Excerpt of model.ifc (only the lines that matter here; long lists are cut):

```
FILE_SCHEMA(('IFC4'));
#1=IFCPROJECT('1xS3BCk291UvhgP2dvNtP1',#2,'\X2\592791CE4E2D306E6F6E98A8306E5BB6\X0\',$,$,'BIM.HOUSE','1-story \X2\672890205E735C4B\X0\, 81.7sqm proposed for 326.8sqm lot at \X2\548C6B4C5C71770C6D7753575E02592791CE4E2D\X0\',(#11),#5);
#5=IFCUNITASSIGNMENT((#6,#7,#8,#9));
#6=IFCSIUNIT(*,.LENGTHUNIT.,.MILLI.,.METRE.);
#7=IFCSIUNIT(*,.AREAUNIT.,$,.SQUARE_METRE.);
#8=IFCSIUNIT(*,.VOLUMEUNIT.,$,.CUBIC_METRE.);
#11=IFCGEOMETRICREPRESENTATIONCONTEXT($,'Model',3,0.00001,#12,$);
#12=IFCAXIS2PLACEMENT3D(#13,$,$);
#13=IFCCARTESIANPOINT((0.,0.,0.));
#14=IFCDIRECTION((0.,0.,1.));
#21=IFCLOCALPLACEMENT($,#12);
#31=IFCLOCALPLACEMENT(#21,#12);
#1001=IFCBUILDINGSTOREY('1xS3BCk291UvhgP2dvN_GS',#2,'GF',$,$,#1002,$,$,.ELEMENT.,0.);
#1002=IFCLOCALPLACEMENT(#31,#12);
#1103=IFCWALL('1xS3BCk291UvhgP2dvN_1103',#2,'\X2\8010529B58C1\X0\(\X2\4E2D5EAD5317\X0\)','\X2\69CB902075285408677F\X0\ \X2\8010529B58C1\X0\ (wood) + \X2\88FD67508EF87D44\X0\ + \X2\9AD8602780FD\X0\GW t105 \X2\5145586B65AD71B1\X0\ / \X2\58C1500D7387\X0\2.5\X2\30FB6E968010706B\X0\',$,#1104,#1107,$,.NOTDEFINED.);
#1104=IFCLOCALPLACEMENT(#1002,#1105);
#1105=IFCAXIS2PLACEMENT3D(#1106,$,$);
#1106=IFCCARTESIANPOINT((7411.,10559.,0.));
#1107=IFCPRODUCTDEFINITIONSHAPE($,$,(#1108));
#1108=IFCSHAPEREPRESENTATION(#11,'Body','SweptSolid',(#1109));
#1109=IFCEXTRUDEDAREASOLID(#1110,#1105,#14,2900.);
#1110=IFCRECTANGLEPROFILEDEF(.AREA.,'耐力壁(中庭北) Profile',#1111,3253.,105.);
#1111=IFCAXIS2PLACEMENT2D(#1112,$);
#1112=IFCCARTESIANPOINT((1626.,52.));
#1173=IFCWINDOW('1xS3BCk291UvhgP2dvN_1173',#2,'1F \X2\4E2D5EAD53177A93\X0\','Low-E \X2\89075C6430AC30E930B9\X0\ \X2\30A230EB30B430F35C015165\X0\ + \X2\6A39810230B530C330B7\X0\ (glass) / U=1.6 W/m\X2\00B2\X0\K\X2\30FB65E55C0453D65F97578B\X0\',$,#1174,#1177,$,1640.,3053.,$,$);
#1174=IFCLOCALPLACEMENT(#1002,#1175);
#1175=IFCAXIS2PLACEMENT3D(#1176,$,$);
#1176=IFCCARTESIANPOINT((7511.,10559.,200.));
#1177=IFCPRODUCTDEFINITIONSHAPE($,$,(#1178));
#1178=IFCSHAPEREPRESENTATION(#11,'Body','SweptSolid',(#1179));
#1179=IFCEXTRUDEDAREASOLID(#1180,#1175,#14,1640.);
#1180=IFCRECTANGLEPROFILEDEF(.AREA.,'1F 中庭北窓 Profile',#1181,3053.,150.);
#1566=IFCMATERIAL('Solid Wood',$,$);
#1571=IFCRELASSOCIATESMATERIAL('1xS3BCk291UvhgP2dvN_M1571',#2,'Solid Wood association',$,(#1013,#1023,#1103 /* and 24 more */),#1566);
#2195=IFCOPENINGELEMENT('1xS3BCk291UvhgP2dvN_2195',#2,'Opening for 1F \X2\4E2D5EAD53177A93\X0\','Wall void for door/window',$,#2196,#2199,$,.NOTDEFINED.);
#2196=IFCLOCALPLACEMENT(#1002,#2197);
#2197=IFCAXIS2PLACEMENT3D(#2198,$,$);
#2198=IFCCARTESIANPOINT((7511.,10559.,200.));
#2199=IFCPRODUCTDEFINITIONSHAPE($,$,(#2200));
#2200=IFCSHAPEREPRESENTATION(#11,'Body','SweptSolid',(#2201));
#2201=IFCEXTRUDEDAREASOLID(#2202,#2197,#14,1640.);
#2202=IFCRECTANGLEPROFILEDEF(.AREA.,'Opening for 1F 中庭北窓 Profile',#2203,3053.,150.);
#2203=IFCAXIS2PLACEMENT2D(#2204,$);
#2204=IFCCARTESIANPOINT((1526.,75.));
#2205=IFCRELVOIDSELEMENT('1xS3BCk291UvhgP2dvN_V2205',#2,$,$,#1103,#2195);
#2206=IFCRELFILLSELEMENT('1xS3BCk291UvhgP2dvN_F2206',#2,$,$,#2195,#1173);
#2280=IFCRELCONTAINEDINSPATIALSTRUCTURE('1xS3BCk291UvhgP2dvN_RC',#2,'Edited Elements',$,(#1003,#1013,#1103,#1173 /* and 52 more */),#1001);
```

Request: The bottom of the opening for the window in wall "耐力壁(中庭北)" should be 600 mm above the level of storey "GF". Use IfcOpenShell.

```python
import numpy as np
import ifcopenshell
import ifcopenshell.api.geometry
import ifcopenshell.geom
import ifcopenshell.util.element
import ifcopenshell.util.placement
import ifcopenshell.util.shape
import ifcopenshell.util.unit

model = ifcopenshell.open("model.ifc")
unit_scale = ifcopenshell.util.unit.calculate_unit_scale(model)

window = model.by_guid("1xS3BCk291UvhgP2dvN_1173")
opening = window.FillsVoids[0].RelatingOpeningElement
storey = ifcopenshell.util.element.get_container(window, ifc_class="IfcBuildingStorey")
level = ifcopenshell.util.placement.get_local_placement(storey.ObjectPlacement)[2, 3]

# The opening's origin need not be at the sill, so measure its lowest point.
shape = ifcopenshell.geom.create_shape(ifcopenshell.geom.settings(), opening)
bottom = ifcopenshell.util.shape.get_shape_bottom_elevation(shape, shape.geometry) / unit_scale
dz = level + 0.6 / unit_scale - bottom

shift = np.array([0.0, 0.0, dz])
# The window is not placed relative to its opening, so move both.
for product in (opening, window):
    matrix = ifcopenshell.util.placement.get_local_placement(product.ObjectPlacement)
    matrix[:3, 3] += shift
    ifcopenshell.api.geometry.edit_object_placement(model, product=product, matrix=matrix, is_si=False)

print(f"moved by {dz * unit_scale:+.3f} m")

model.write("model_v2.ifc")
```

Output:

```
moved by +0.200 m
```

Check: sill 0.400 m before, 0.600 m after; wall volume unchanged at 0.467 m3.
